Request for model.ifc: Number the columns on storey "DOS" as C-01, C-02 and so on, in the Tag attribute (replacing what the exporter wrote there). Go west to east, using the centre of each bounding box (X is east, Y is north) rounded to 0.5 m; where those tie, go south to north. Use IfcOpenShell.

First a look at what the model holds.

```python
import ifcopenshell
import ifcopenshell.util.element
import ifcopenshell.util.placement

model = ifcopenshell.open("model.ifc")
print(model.schema)
storey = next(s for s in model.by_type("IfcBuildingStorey") if s.Name == "DOS")
columns = [e for e in ifcopenshell.util.element.get_decomposition(storey) if e.is_a("IfcColumn")]
for e in sorted(columns, key=lambda e: e.id()):
    origin = ifcopenshell.util.placement.get_local_placement(e.ObjectPlacement)[:3, 3]
    print(e.id(), e.Tag, e.Name, origin.round(2) + 0.0, sep=" | ")
```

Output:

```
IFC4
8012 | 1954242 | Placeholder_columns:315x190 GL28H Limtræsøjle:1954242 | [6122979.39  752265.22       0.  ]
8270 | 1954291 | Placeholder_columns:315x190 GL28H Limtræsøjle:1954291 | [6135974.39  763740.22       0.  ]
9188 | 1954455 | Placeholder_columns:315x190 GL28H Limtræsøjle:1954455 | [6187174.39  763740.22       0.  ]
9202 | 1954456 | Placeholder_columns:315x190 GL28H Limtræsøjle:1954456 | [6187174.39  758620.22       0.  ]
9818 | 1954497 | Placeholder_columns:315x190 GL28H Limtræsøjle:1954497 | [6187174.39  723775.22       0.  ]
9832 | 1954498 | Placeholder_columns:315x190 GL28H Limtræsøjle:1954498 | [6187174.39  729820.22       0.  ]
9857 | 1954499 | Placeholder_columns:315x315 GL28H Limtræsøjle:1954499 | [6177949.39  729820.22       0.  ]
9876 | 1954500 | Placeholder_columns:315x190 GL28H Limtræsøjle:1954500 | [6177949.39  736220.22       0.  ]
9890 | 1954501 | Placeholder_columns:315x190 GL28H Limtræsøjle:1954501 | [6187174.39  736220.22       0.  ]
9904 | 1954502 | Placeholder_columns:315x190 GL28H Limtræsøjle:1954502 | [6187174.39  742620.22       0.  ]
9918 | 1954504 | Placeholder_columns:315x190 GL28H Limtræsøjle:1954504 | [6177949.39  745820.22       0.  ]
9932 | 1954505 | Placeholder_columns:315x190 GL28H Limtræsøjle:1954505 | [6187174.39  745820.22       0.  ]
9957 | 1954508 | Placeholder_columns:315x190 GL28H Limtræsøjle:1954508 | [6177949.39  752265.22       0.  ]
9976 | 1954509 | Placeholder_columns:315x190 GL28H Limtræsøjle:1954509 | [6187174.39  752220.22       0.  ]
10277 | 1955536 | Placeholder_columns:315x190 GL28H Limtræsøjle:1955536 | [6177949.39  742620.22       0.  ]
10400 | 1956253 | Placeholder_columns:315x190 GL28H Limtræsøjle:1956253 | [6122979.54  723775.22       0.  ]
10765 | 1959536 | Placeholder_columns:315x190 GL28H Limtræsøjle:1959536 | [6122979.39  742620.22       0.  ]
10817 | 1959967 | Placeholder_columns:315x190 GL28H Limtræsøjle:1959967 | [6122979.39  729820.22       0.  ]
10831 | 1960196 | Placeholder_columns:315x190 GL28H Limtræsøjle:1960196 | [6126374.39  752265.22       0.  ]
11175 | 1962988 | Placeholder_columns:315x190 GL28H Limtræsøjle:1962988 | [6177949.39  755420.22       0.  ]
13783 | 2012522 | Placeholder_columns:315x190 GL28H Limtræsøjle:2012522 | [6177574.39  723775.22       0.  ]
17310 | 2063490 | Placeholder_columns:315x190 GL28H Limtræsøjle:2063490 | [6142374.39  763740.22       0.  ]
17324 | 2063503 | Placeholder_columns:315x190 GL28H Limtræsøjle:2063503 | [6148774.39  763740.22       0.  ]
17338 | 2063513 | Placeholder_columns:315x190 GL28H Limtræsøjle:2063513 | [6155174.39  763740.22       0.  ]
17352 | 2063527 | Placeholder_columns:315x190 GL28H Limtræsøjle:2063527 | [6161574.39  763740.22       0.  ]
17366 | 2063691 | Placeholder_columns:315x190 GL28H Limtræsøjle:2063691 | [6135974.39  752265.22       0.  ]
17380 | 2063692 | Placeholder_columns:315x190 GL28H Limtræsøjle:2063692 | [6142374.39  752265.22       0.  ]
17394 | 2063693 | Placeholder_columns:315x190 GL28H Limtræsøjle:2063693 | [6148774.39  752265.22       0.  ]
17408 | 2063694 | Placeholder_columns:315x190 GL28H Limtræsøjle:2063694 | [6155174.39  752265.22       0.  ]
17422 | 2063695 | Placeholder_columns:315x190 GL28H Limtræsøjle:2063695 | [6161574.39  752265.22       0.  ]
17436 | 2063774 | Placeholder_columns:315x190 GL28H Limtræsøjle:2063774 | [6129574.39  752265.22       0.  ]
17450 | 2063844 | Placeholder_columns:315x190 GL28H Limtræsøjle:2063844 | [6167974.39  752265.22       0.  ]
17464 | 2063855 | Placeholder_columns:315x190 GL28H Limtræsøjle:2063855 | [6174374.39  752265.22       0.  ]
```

```python
import ifcopenshell
import ifcopenshell.geom
import ifcopenshell.util.element
import ifcopenshell.util.shape

model = ifcopenshell.open("model.ifc")
settings = ifcopenshell.geom.settings()
settings.set("use-world-coords", True)


def centre(element):
    shape = ifcopenshell.geom.create_shape(settings, element)
    return ifcopenshell.util.shape.get_bbox_centroid(shape.geometry)


storey = next(s for s in model.by_type("IfcBuildingStorey") if s.Name == "DOS")
columns = [e for e in ifcopenshell.util.element.get_decomposition(storey) if e.is_a("IfcColumn")]

# Insertion points can sit at a corner or the storey origin, so sort by the geometry (in metres).
centres = {e: centre(e) for e in columns}
columns.sort(key=lambda e: (round(centres[e][0] / 0.5), centres[e][1]))

for i, e in enumerate(columns, start=1):
    number = f"C-{i:02d}"
    e.Tag = number
    print(e.id(), number)

model.write("model-out.ifc")
```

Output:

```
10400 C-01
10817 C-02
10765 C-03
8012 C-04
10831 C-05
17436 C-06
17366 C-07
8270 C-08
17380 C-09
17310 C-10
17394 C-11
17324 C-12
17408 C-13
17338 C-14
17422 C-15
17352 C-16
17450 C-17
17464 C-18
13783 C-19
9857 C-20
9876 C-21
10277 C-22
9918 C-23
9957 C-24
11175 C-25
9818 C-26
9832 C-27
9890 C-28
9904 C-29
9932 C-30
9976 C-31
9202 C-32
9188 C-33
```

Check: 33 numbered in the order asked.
